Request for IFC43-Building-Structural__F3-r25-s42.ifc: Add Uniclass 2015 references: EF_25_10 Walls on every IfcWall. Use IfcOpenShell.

First a look at what the model holds.

```python
import ifcopenshell

model = ifcopenshell.open("IFC43-Building-Structural__F3-r25-s42.ifc")
print(model.schema)
print("classifications:", [c.Name for c in model.by_type("IfcClassification")])
for ifc_class in ("IfcDoor", "IfcRoof", "IfcStair", "IfcWall", "IfcWindow"):
    print(ifc_class, len(model.by_type(ifc_class)))
```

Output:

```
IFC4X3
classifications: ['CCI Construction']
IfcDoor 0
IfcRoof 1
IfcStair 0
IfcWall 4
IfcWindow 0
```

```python
import ifcopenshell
import ifcopenshell.api.classification

model = ifcopenshell.open("IFC43-Building-Structural__F3-r25-s42.ifc")

system = ifcopenshell.api.classification.add_classification(model, classification="Uniclass 2015")

codes = {
    "IfcWall": ("EF_25_10", "Walls"),
}
for ifc_class, (code, name) in codes.items():
    products = model.by_type(ifc_class)
    ifcopenshell.api.classification.add_reference(
        model, products=products, classification=system, identification=code, name=name
    )
    print(code, len(products))

model.write("IFC43-Building-Structural__F3-r25-s42_edited.ifc")
```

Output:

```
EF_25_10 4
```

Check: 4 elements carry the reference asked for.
